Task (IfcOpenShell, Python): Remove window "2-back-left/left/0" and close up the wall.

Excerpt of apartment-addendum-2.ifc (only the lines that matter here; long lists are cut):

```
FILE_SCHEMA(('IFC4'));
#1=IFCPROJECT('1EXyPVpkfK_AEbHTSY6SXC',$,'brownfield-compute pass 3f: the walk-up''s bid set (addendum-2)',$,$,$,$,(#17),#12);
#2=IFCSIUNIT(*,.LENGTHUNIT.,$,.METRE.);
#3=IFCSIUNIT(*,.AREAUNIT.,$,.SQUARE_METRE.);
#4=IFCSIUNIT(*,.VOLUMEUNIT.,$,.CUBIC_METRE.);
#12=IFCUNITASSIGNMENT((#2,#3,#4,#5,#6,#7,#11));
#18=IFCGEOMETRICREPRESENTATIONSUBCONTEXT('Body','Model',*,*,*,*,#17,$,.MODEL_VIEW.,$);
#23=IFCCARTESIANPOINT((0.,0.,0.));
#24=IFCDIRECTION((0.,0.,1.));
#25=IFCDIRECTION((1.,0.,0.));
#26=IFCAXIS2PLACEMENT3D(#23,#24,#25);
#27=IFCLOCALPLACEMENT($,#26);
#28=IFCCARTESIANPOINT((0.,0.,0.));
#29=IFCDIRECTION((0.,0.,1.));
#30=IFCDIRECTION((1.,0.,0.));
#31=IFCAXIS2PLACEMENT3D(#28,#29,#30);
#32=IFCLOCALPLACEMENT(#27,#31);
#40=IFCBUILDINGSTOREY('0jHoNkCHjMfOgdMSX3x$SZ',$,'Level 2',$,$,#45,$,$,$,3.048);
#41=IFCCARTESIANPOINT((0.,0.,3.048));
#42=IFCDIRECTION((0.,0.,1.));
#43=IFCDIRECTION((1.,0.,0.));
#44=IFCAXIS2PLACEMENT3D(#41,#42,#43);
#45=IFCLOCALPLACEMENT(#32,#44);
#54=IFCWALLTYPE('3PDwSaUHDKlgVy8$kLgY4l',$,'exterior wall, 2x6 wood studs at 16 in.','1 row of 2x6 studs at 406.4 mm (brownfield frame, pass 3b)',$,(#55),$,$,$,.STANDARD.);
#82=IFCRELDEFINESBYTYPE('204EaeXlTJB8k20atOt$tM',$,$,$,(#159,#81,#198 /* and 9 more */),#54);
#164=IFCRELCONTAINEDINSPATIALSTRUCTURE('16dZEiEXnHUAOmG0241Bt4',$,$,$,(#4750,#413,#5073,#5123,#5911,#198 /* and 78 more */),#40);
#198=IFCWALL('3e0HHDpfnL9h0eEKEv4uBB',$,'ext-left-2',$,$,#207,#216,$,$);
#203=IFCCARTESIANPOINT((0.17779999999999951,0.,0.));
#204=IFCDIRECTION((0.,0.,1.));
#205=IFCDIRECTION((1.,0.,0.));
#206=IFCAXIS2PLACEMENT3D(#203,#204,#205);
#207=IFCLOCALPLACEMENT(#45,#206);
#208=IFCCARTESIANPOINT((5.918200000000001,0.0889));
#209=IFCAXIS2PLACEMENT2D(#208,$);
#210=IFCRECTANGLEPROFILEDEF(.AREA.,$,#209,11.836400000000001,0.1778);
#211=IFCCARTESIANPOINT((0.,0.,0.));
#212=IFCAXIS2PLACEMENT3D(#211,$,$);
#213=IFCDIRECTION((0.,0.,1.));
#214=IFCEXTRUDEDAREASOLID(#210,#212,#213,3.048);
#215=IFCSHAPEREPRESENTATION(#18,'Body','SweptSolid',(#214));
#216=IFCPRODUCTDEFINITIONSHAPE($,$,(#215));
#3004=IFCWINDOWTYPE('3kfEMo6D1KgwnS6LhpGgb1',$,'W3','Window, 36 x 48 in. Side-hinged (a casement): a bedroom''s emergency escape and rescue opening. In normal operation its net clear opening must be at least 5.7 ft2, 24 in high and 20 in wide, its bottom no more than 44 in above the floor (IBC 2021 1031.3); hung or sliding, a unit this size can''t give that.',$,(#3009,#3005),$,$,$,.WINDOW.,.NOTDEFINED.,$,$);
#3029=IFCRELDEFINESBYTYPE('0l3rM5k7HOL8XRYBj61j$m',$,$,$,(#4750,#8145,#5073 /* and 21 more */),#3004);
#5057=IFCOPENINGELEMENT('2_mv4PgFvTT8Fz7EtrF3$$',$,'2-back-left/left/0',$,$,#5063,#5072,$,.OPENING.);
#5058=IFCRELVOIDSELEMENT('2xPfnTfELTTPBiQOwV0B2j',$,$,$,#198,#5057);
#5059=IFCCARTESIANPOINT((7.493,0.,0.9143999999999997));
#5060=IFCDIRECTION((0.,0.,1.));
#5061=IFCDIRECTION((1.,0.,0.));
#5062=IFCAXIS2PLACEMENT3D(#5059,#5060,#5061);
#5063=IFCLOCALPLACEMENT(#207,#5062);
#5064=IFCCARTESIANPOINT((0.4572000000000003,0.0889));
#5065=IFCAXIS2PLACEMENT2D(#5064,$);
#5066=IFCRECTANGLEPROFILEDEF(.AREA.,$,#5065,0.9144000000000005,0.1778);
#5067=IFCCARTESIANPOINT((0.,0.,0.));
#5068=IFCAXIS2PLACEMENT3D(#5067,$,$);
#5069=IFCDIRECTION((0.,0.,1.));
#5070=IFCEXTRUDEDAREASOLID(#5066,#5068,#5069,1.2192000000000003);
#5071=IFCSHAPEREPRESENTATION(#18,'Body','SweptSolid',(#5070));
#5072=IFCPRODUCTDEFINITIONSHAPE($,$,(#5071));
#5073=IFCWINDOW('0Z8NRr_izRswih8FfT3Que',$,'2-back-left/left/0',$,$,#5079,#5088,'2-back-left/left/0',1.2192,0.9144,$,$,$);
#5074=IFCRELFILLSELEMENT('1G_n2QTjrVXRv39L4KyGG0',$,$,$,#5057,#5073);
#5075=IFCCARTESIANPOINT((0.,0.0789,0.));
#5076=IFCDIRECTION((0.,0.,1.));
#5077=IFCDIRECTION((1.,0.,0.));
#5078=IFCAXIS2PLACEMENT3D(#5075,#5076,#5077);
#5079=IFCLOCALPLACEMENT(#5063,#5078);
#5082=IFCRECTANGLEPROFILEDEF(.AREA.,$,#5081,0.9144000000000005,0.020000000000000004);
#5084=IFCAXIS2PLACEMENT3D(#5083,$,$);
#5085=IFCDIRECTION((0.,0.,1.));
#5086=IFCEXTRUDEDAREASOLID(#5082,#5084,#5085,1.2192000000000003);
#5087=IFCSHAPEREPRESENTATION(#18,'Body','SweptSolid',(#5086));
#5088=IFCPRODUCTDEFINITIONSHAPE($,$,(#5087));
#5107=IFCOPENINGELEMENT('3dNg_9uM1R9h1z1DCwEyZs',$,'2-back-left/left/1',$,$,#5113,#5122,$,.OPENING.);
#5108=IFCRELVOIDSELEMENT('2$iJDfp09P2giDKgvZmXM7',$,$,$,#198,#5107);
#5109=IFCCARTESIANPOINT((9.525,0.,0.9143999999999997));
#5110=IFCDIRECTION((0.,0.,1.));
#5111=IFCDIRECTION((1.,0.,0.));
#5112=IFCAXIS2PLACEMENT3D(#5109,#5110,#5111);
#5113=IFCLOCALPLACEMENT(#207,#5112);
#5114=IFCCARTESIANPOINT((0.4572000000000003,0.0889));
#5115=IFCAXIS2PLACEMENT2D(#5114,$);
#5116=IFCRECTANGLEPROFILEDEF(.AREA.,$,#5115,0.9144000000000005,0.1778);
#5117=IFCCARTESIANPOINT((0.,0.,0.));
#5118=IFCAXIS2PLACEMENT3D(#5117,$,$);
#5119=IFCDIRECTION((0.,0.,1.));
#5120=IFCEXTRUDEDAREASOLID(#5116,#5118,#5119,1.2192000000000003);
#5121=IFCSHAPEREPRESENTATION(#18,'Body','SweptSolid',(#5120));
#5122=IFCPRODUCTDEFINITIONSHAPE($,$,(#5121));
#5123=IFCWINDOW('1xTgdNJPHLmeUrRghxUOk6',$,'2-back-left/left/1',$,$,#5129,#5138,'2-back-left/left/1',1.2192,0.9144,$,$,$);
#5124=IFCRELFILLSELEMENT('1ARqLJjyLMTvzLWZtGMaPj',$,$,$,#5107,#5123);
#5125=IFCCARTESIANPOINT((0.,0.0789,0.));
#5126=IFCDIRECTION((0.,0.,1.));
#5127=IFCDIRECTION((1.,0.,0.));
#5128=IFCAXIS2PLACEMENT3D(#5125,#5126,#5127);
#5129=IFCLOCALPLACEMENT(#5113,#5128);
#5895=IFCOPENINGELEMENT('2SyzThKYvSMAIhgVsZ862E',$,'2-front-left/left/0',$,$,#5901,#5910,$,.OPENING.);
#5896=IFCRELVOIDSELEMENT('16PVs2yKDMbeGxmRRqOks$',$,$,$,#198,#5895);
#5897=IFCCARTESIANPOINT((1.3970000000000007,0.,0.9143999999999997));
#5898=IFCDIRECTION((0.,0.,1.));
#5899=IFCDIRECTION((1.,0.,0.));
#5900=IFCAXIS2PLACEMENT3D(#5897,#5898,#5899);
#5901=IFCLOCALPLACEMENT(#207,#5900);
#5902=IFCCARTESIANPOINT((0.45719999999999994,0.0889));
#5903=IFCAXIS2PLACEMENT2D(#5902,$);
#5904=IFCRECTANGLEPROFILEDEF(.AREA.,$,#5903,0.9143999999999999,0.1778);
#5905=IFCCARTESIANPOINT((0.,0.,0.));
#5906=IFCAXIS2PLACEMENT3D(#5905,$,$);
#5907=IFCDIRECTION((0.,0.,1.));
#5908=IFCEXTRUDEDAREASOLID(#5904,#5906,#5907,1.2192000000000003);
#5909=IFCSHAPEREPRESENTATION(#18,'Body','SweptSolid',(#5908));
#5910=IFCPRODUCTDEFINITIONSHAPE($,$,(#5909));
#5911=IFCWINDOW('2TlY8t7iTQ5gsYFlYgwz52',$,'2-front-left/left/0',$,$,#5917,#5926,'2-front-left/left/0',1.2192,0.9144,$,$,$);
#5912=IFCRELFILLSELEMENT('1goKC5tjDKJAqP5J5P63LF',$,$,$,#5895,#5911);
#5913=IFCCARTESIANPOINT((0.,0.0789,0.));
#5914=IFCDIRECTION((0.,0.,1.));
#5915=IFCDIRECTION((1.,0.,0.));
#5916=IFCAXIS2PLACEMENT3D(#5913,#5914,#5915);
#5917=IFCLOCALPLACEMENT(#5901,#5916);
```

```python
import ifcopenshell
import ifcopenshell.api.feature
import ifcopenshell.api.root
import ifcopenshell.geom
import ifcopenshell.util.shape

model = ifcopenshell.open("apartment-addendum-2.ifc")
settings = ifcopenshell.geom.settings()


def volume(element):
    """Net volume in cubic metres, openings subtracted."""
    shape = ifcopenshell.geom.create_shape(settings, element)
    return ifcopenshell.util.shape.get_volume(shape.geometry)


window = model.by_guid("0Z8NRr_izRswih8FfT3Que")
opening = window.FillsVoids[0].RelatingOpeningElement
wall = opening.VoidsElements[0].RelatingBuildingElement
before = volume(wall)

ifcopenshell.api.root.remove_product(model, product=window)
ifcopenshell.api.feature.remove_feature(model, feature=opening)

after = volume(wall)

print(f"wall volume {before:.3f} -> {after:.3f} m3")

model.write("apartment-addendum-2-out.ifc")
```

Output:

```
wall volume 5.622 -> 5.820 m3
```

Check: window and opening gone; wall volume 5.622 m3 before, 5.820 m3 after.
